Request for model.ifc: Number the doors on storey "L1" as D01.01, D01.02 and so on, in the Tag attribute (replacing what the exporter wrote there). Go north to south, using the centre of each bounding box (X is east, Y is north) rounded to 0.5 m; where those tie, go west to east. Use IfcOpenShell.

First a look at what the model holds.

```python
import ifcopenshell
import ifcopenshell.util.element
import ifcopenshell.util.placement

model = ifcopenshell.open("model.ifc")
print(model.schema)
storey = next(s for s in model.by_type("IfcBuildingStorey") if s.Name == "L1")
doors = [e for e in ifcopenshell.util.element.get_decomposition(storey) if e.is_a("IfcDoor")]
for e in sorted(doors, key=lambda e: e.id()):
    origin = ifcopenshell.util.placement.get_local_placement(e.ObjectPlacement)[:3, 3]
    print(e.id(), e.Tag, e.Name, origin.round(2) + 0.0, sep=" | ")
```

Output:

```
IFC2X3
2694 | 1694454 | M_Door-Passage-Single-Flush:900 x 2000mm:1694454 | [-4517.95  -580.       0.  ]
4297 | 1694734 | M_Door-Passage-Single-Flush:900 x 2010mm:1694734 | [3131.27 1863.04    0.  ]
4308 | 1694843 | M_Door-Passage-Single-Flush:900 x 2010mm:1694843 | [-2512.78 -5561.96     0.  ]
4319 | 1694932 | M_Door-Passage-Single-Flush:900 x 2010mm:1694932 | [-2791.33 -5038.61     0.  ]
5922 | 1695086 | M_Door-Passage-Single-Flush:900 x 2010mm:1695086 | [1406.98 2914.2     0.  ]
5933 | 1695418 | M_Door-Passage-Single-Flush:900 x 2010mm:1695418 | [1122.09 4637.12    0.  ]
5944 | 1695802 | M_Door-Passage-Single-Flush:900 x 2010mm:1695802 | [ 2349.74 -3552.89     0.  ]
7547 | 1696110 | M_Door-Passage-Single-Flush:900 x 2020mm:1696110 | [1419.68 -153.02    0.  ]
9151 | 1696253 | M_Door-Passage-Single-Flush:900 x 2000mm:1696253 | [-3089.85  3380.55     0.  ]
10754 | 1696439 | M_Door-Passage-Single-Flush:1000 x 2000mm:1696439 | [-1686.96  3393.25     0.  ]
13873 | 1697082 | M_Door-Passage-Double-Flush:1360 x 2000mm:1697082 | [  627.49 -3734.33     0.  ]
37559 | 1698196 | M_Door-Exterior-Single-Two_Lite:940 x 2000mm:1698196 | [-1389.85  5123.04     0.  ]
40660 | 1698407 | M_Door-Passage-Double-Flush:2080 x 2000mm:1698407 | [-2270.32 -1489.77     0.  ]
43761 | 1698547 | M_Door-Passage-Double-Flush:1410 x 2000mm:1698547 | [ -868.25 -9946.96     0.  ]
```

```python
import ifcopenshell
import ifcopenshell.geom
import ifcopenshell.util.element
import ifcopenshell.util.shape

model = ifcopenshell.open("model.ifc")
settings = ifcopenshell.geom.settings()
settings.set("use-world-coords", True)


def centre(element):
    shape = ifcopenshell.geom.create_shape(settings, element)
    return ifcopenshell.util.shape.get_bbox_centroid(shape.geometry)


storey = next(s for s in model.by_type("IfcBuildingStorey") if s.Name == "L1")
doors = [e for e in ifcopenshell.util.element.get_decomposition(storey) if e.is_a("IfcDoor")]

# Insertion points can sit at a corner or the storey origin, so sort by the geometry (in metres).
centres = {e: centre(e) for e in doors}
doors.sort(key=lambda e: (-round(centres[e][1] / 0.5), centres[e][0]))

for i, e in enumerate(doors, start=1):
    number = f"D01.{i:02d}"
    e.Tag = number
    print(e.id(), number)

model.write("model_v2.ifc")
```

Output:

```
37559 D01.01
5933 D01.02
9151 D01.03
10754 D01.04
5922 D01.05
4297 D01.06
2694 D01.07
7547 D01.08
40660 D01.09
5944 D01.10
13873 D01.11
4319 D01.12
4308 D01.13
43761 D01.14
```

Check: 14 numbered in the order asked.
